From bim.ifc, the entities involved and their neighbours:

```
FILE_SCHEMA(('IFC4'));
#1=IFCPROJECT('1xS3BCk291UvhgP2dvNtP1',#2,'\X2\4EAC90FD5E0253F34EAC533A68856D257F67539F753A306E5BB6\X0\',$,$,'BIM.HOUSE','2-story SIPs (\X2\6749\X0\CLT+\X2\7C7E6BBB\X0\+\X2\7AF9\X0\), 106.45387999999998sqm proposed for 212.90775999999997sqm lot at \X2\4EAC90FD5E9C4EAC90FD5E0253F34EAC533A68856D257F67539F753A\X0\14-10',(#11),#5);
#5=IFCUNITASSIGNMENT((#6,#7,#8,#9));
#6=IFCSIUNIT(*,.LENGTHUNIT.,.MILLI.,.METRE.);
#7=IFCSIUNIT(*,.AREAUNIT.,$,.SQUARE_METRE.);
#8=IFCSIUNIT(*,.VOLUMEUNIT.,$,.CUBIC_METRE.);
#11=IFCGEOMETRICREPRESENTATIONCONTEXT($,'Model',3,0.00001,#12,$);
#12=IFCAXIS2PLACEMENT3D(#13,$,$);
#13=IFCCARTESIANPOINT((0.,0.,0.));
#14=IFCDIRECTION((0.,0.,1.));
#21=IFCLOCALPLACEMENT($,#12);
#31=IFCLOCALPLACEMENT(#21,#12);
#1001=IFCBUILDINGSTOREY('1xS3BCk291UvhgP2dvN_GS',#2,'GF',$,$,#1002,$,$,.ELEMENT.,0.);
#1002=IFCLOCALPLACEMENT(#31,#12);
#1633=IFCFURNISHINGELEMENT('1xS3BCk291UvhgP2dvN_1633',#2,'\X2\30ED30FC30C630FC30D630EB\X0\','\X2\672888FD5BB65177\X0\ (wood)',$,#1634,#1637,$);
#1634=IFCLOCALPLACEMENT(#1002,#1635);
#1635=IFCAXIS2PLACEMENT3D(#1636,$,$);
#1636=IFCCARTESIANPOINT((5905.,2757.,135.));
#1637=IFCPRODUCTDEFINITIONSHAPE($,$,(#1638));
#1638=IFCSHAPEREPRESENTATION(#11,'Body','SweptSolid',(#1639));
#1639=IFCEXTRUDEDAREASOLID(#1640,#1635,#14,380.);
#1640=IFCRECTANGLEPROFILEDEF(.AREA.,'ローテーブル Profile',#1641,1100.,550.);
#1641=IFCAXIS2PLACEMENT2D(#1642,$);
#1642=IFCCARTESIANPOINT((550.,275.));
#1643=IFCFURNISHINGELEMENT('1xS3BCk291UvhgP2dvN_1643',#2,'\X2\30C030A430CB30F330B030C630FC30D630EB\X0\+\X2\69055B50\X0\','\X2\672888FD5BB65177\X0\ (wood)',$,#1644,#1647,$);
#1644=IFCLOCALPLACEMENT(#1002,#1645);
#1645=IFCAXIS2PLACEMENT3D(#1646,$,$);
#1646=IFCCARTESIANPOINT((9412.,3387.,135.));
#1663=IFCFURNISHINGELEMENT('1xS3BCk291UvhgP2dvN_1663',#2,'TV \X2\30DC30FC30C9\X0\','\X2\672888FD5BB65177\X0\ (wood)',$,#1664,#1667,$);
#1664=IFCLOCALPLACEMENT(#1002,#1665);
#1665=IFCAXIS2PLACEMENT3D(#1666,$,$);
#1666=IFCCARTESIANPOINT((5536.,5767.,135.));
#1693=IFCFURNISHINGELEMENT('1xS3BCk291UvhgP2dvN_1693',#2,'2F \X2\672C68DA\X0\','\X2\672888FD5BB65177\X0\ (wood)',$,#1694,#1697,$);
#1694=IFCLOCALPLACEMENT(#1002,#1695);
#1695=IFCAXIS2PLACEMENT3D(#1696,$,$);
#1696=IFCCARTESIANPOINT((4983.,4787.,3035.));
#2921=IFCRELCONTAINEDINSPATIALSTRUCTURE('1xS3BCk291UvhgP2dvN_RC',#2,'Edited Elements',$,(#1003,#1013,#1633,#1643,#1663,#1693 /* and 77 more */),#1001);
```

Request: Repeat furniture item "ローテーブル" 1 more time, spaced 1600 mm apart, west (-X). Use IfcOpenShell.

```python
import numpy as np
import ifcopenshell
import ifcopenshell.api.geometry
import ifcopenshell.api.root
import ifcopenshell.util.element
import ifcopenshell.util.placement
import ifcopenshell.util.unit

model = ifcopenshell.open("bim.ifc")
unit_scale = ifcopenshell.util.unit.calculate_unit_scale(model)


def reuse_history(source, copy):
    """copy_class also copies each property set's owner history, people and application; keep the originals."""
    for rel in copy.IsDefinedBy:
        if rel.is_a("IfcRelDefinesByProperties") and (history := rel.RelatingPropertyDefinition.OwnerHistory):
            rel.RelatingPropertyDefinition.OwnerHistory = source.OwnerHistory
            ifcopenshell.util.element.remove_deep2(model, history)


source = model.by_guid("1xS3BCk291UvhgP2dvN_1633")
base = ifcopenshell.util.placement.get_local_placement(source.ObjectPlacement)
step = np.array([-1.0, 0.0, 0.0]) * 1.6 / unit_scale

for i in range(1, 2):
    copy = ifcopenshell.api.root.copy_class(model, product=source)
    copy.Representation = ifcopenshell.util.element.copy_deep(
        model, source.Representation, exclude=["IfcGeometricRepresentationContext", "IfcRepresentationMap"]
    )
    reuse_history(source, copy)
    matrix = base.copy()
    matrix[:3, 3] += i * step
    print("added at", matrix[:3, 3].round(3) + 0.0)
    ifcopenshell.api.geometry.edit_object_placement(model, product=copy, matrix=matrix, is_si=False)

model.write("bim-out.ifc")
```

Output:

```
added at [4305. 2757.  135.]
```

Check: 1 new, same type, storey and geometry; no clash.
